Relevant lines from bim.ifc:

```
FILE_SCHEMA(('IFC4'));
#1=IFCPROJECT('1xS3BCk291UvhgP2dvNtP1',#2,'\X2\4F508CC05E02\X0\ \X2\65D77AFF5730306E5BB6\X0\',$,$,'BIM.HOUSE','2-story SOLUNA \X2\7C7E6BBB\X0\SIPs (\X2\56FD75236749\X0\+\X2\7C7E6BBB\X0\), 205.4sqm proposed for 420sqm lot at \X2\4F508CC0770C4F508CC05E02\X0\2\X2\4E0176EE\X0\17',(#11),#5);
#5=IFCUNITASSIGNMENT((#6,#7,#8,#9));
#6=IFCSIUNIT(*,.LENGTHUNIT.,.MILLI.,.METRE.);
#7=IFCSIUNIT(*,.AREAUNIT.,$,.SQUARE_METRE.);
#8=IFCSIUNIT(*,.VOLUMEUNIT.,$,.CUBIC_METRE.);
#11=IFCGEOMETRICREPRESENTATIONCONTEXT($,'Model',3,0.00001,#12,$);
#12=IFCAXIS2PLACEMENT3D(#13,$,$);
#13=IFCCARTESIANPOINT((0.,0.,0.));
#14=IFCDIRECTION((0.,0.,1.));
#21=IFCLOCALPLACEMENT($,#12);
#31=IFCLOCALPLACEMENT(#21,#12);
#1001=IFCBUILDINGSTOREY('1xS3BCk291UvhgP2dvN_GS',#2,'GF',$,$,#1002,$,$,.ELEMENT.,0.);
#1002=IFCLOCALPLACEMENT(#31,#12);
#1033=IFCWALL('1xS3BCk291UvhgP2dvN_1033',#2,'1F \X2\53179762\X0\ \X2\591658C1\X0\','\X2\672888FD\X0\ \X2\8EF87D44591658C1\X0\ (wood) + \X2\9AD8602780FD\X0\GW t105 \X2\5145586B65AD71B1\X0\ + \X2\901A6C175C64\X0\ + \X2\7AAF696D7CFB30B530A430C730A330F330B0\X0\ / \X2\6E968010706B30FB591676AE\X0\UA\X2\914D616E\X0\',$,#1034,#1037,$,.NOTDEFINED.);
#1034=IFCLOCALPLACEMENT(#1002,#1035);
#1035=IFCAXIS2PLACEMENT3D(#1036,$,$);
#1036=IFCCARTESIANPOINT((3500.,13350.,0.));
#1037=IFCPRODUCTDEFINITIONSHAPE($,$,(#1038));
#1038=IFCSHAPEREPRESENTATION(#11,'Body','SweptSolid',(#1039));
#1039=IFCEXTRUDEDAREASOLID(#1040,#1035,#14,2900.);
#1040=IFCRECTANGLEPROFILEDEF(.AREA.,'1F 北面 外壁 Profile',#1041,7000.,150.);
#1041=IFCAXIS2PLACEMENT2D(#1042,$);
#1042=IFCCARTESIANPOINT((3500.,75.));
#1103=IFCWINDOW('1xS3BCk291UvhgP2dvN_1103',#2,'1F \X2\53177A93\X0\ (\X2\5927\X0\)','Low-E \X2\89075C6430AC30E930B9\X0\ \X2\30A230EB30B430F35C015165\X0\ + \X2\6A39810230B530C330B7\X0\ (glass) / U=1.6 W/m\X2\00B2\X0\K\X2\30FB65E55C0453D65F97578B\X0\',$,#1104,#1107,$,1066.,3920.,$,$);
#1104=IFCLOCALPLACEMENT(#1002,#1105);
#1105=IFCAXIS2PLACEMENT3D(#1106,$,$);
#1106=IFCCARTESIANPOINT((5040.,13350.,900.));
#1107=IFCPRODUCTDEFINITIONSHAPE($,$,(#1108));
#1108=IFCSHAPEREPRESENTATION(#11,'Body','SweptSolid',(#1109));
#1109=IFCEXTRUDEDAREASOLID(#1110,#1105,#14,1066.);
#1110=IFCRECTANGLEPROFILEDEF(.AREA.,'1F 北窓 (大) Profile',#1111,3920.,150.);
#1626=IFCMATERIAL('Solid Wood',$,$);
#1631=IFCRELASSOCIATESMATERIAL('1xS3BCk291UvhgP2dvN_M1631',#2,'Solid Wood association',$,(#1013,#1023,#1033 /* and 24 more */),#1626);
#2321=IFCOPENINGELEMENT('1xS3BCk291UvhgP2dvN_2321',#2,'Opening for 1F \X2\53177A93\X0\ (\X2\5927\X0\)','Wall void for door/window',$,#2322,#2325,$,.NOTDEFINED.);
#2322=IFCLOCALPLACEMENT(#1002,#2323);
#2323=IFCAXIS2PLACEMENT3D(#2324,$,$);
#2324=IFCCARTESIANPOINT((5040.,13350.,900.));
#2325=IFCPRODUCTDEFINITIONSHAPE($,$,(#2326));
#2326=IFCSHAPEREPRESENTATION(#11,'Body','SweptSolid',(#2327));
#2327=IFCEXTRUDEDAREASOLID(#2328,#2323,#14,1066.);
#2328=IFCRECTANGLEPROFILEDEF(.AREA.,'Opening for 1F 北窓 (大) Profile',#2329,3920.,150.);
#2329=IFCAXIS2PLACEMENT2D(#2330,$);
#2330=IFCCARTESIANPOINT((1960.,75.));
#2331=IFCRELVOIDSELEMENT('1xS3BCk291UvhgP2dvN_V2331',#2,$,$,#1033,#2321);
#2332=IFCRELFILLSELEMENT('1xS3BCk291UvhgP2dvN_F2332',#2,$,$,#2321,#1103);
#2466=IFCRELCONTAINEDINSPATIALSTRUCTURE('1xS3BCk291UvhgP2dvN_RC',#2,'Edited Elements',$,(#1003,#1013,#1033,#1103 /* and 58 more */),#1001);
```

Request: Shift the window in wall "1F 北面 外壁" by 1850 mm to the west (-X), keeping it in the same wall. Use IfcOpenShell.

```python
import ifcopenshell
import ifcopenshell.api.geometry
import ifcopenshell.util.placement

model = ifcopenshell.open("bim.ifc")

window = model.by_guid("1xS3BCk291UvhgP2dvN_1103")
opening = window.FillsVoids[0].RelatingOpeningElement
wall = opening.VoidsElements[0].RelatingBuildingElement

wall_matrix = ifcopenshell.util.placement.get_local_placement(wall.ObjectPlacement)
shift = wall_matrix[:3, 0] * -1850.0
before = ifcopenshell.util.placement.get_local_placement(window.ObjectPlacement)[:3, 3].copy()

# The window is not placed relative to its opening, so move both.
for product in (opening, window):
    matrix = ifcopenshell.util.placement.get_local_placement(product.ObjectPlacement)
    matrix[:3, 3] += shift
    ifcopenshell.api.geometry.edit_object_placement(model, product=product, matrix=matrix, is_si=False)

after = ifcopenshell.util.placement.get_local_placement(window.ObjectPlacement)[:3, 3]
print("window moved by", (after - before).round(3) + 0.0)

model.write("bim_v2.ifc")
```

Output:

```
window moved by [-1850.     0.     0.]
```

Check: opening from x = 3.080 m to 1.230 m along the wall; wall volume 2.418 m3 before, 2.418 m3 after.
